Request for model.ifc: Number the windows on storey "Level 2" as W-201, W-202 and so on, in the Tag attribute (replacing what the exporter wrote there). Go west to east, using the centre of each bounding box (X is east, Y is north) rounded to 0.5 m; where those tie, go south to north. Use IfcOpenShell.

First a look at what the model holds.

```python
import ifcopenshell
import ifcopenshell.util.element
import ifcopenshell.util.placement

model = ifcopenshell.open("model.ifc")
print(model.schema)
storey = next(s for s in model.by_type("IfcBuildingStorey") if s.Name == "Level 2")
windows = [e for e in ifcopenshell.util.element.get_decomposition(storey) if e.is_a("IfcWindow")]
for e in sorted(windows, key=lambda e: e.id()):
    origin = ifcopenshell.util.placement.get_local_placement(e.ObjectPlacement)[:3, 3]
    print(e.id(), e.Tag, e.Name, origin.round(2) + 0.0, sep=" | ")
```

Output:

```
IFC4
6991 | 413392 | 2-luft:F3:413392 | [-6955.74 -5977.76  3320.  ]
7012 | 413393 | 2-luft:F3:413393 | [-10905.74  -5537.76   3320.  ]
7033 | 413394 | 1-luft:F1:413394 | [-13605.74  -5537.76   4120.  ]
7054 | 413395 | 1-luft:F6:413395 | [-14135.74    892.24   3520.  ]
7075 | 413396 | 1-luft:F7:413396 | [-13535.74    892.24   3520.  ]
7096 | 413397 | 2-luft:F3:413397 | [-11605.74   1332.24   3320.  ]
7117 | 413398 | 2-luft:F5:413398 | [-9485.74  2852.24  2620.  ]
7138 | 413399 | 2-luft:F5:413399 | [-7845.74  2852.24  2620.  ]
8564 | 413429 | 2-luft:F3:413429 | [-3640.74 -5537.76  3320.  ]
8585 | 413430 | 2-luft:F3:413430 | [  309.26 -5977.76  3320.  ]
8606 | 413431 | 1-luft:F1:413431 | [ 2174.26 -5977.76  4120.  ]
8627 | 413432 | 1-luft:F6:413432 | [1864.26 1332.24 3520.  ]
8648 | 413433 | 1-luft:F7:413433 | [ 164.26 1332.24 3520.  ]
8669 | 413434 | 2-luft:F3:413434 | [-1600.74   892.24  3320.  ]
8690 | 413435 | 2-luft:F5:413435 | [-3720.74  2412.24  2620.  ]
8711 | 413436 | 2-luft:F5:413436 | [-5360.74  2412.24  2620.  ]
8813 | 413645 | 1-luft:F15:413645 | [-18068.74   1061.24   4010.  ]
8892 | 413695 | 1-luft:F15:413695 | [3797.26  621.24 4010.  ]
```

```python
import ifcopenshell
import ifcopenshell.geom
import ifcopenshell.util.element
import ifcopenshell.util.shape

model = ifcopenshell.open("model.ifc")
settings = ifcopenshell.geom.settings()
settings.set("use-world-coords", True)


def centre(element):
    shape = ifcopenshell.geom.create_shape(settings, element)
    return ifcopenshell.util.shape.get_bbox_centroid(shape.geometry)


storey = next(s for s in model.by_type("IfcBuildingStorey") if s.Name == "Level 2")
windows = [e for e in ifcopenshell.util.element.get_decomposition(storey) if e.is_a("IfcWindow")]

# Insertion points can sit at a corner or the storey origin, so sort by the geometry (in metres).
centres = {e: centre(e) for e in windows}
windows.sort(key=lambda e: (round(centres[e][0] / 0.5), centres[e][1]))

for i, e in enumerate(windows, start=1):
    number = f"W-2{i:02d}"
    e.Tag = number
    print(e.id(), number)

model.write("model_v2.ifc")
```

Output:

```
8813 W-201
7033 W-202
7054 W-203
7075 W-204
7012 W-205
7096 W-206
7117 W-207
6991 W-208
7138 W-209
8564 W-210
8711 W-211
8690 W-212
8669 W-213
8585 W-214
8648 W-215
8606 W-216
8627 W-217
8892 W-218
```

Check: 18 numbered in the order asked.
